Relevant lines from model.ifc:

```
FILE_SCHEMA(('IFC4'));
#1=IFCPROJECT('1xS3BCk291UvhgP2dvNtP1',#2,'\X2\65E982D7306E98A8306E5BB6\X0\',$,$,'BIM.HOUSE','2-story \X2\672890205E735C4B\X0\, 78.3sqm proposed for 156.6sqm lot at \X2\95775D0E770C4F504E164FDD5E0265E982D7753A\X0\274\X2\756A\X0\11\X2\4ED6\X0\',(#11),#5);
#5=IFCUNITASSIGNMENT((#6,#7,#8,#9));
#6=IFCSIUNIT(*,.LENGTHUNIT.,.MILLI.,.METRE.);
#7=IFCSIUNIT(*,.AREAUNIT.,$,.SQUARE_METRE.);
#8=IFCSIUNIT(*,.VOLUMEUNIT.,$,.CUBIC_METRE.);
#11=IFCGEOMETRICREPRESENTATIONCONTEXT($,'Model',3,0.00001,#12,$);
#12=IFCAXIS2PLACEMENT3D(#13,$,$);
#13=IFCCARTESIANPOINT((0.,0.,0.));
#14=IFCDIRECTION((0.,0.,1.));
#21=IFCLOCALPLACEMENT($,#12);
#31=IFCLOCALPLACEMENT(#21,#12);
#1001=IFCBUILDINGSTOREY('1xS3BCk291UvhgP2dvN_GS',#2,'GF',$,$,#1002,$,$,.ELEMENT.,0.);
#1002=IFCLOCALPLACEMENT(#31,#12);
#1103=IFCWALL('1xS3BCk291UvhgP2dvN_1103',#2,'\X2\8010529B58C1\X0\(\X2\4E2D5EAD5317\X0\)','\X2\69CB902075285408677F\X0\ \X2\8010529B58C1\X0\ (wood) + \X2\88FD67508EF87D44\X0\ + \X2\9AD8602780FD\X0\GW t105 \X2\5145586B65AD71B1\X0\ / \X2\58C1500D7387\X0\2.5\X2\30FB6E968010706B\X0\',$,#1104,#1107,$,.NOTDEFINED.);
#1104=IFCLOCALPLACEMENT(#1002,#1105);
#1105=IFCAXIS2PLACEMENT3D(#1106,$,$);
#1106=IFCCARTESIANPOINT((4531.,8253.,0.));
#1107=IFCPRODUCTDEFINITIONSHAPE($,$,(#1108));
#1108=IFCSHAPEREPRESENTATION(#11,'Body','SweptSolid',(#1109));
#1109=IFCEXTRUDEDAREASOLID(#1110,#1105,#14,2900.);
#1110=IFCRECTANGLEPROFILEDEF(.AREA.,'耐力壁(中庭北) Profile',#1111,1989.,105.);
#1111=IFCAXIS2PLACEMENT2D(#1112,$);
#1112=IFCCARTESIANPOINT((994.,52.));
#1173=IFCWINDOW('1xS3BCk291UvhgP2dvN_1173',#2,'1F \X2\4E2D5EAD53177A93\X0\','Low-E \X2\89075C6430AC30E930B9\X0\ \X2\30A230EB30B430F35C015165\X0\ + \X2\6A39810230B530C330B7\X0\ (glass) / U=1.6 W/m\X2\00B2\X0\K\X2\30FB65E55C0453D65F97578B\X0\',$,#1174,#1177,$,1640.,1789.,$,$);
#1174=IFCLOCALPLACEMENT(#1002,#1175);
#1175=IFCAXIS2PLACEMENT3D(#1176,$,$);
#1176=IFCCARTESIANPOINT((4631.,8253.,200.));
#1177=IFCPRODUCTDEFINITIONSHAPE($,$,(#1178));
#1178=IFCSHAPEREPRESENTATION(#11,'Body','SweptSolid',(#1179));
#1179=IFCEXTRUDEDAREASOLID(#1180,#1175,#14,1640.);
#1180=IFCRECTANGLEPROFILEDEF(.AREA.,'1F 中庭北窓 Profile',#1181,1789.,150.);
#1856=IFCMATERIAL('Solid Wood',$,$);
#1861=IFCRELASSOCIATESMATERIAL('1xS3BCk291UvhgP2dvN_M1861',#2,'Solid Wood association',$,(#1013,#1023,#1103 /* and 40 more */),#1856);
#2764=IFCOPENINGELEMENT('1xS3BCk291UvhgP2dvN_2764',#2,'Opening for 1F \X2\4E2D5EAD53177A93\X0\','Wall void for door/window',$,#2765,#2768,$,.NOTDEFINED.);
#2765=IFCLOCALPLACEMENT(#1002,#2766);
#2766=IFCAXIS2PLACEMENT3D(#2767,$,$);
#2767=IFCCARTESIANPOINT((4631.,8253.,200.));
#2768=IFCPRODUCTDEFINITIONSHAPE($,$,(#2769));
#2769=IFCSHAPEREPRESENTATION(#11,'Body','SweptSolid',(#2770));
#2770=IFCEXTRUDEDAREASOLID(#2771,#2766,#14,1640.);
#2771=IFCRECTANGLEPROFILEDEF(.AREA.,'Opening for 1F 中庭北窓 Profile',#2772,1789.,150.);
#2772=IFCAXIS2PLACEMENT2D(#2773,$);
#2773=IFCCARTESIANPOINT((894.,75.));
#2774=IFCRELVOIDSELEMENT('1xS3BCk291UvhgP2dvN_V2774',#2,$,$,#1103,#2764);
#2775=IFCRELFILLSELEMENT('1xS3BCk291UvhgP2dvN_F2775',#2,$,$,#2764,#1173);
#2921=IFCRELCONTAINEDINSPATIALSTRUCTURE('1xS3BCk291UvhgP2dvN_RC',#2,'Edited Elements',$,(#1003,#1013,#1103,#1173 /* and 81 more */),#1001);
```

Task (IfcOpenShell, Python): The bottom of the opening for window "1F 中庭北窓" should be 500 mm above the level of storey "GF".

```python
import numpy as np
import ifcopenshell
import ifcopenshell.api.geometry
import ifcopenshell.geom
import ifcopenshell.util.element
import ifcopenshell.util.placement
import ifcopenshell.util.shape
import ifcopenshell.util.unit

model = ifcopenshell.open("model.ifc")
unit_scale = ifcopenshell.util.unit.calculate_unit_scale(model)

window = model.by_id(1173)
opening = window.FillsVoids[0].RelatingOpeningElement
storey = ifcopenshell.util.element.get_container(window, ifc_class="IfcBuildingStorey")
level = ifcopenshell.util.placement.get_local_placement(storey.ObjectPlacement)[2, 3]

# The opening's origin need not be at the sill, so measure its lowest point.
shape = ifcopenshell.geom.create_shape(ifcopenshell.geom.settings(), opening)
bottom = ifcopenshell.util.shape.get_shape_bottom_elevation(shape, shape.geometry) / unit_scale
dz = level + 0.5 / unit_scale - bottom

shift = np.array([0.0, 0.0, dz])
# The window is not placed relative to its opening, so move both.
for product in (opening, window):
    matrix = ifcopenshell.util.placement.get_local_placement(product.ObjectPlacement)
    matrix[:3, 3] += shift
    ifcopenshell.api.geometry.edit_object_placement(model, product=product, matrix=matrix, is_si=False)

print(f"moved by {dz * unit_scale:+.3f} m")

model.write("model_rev.ifc")
```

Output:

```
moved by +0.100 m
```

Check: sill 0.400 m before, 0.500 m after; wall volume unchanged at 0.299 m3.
